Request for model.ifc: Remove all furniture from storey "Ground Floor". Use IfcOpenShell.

First a look at what the model holds.

```python
import ifcopenshell
import ifcopenshell.util.element

model = ifcopenshell.open("model.ifc")
print(model.schema)
storey = next(s for s in model.by_type("IfcBuildingStorey") if s.Name == "Ground Floor")
furniture = [e for e in ifcopenshell.util.element.get_decomposition(storey) if e.is_a("IfcFurnishingElement")]
seen = {}
for e in furniture:
    element_type = ifcopenshell.util.element.get_type(e)
    name = element_type.Name if element_type not in (None, e) else None
    seen[name] = seen.get(name, 0) + 1
for name, count in sorted(seen.items(), key=str):
    print(count, "x", name)
```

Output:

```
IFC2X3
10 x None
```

```python
import ifcopenshell
import ifcopenshell.api.root
import ifcopenshell.util.element

model = ifcopenshell.open("model.ifc")

storey = next(s for s in model.by_type("IfcBuildingStorey") if s.Name == "Ground Floor")
furniture = [e for e in ifcopenshell.util.element.get_decomposition(storey) if e.is_a("IfcFurnishingElement")]

for e in furniture:
    ifcopenshell.api.root.remove_product(model, product=e)
print(len(furniture), "removed")

model.write("model-out.ifc")
```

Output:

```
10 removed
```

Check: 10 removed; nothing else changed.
